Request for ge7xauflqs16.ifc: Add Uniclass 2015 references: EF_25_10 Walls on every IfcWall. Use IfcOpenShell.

First a look at what the model holds.

```python
import ifcopenshell

model = ifcopenshell.open("ge7xauflqs16.ifc")
print(model.schema)
print("classifications:", [c.Name for c in model.by_type("IfcClassification")])
for ifc_class in ("IfcDoor", "IfcRoof", "IfcStair", "IfcWall", "IfcWindow"):
    print(ifc_class, len(model.by_type(ifc_class)))
```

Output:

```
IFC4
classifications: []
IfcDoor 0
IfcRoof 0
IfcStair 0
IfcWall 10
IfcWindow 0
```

```python
import ifcopenshell
import ifcopenshell.api.classification

model = ifcopenshell.open("ge7xauflqs16.ifc")

system = ifcopenshell.api.classification.add_classification(model, classification="Uniclass 2015")

codes = {
    "IfcWall": ("EF_25_10", "Walls"),
}
for ifc_class, (code, name) in codes.items():
    products = model.by_type(ifc_class)
    ifcopenshell.api.classification.add_reference(
        model, products=products, classification=system, identification=code, name=name
    )
    print(code, len(products))

model.write("ge7xauflqs16_updated.ifc")
```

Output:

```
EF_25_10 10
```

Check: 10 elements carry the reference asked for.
